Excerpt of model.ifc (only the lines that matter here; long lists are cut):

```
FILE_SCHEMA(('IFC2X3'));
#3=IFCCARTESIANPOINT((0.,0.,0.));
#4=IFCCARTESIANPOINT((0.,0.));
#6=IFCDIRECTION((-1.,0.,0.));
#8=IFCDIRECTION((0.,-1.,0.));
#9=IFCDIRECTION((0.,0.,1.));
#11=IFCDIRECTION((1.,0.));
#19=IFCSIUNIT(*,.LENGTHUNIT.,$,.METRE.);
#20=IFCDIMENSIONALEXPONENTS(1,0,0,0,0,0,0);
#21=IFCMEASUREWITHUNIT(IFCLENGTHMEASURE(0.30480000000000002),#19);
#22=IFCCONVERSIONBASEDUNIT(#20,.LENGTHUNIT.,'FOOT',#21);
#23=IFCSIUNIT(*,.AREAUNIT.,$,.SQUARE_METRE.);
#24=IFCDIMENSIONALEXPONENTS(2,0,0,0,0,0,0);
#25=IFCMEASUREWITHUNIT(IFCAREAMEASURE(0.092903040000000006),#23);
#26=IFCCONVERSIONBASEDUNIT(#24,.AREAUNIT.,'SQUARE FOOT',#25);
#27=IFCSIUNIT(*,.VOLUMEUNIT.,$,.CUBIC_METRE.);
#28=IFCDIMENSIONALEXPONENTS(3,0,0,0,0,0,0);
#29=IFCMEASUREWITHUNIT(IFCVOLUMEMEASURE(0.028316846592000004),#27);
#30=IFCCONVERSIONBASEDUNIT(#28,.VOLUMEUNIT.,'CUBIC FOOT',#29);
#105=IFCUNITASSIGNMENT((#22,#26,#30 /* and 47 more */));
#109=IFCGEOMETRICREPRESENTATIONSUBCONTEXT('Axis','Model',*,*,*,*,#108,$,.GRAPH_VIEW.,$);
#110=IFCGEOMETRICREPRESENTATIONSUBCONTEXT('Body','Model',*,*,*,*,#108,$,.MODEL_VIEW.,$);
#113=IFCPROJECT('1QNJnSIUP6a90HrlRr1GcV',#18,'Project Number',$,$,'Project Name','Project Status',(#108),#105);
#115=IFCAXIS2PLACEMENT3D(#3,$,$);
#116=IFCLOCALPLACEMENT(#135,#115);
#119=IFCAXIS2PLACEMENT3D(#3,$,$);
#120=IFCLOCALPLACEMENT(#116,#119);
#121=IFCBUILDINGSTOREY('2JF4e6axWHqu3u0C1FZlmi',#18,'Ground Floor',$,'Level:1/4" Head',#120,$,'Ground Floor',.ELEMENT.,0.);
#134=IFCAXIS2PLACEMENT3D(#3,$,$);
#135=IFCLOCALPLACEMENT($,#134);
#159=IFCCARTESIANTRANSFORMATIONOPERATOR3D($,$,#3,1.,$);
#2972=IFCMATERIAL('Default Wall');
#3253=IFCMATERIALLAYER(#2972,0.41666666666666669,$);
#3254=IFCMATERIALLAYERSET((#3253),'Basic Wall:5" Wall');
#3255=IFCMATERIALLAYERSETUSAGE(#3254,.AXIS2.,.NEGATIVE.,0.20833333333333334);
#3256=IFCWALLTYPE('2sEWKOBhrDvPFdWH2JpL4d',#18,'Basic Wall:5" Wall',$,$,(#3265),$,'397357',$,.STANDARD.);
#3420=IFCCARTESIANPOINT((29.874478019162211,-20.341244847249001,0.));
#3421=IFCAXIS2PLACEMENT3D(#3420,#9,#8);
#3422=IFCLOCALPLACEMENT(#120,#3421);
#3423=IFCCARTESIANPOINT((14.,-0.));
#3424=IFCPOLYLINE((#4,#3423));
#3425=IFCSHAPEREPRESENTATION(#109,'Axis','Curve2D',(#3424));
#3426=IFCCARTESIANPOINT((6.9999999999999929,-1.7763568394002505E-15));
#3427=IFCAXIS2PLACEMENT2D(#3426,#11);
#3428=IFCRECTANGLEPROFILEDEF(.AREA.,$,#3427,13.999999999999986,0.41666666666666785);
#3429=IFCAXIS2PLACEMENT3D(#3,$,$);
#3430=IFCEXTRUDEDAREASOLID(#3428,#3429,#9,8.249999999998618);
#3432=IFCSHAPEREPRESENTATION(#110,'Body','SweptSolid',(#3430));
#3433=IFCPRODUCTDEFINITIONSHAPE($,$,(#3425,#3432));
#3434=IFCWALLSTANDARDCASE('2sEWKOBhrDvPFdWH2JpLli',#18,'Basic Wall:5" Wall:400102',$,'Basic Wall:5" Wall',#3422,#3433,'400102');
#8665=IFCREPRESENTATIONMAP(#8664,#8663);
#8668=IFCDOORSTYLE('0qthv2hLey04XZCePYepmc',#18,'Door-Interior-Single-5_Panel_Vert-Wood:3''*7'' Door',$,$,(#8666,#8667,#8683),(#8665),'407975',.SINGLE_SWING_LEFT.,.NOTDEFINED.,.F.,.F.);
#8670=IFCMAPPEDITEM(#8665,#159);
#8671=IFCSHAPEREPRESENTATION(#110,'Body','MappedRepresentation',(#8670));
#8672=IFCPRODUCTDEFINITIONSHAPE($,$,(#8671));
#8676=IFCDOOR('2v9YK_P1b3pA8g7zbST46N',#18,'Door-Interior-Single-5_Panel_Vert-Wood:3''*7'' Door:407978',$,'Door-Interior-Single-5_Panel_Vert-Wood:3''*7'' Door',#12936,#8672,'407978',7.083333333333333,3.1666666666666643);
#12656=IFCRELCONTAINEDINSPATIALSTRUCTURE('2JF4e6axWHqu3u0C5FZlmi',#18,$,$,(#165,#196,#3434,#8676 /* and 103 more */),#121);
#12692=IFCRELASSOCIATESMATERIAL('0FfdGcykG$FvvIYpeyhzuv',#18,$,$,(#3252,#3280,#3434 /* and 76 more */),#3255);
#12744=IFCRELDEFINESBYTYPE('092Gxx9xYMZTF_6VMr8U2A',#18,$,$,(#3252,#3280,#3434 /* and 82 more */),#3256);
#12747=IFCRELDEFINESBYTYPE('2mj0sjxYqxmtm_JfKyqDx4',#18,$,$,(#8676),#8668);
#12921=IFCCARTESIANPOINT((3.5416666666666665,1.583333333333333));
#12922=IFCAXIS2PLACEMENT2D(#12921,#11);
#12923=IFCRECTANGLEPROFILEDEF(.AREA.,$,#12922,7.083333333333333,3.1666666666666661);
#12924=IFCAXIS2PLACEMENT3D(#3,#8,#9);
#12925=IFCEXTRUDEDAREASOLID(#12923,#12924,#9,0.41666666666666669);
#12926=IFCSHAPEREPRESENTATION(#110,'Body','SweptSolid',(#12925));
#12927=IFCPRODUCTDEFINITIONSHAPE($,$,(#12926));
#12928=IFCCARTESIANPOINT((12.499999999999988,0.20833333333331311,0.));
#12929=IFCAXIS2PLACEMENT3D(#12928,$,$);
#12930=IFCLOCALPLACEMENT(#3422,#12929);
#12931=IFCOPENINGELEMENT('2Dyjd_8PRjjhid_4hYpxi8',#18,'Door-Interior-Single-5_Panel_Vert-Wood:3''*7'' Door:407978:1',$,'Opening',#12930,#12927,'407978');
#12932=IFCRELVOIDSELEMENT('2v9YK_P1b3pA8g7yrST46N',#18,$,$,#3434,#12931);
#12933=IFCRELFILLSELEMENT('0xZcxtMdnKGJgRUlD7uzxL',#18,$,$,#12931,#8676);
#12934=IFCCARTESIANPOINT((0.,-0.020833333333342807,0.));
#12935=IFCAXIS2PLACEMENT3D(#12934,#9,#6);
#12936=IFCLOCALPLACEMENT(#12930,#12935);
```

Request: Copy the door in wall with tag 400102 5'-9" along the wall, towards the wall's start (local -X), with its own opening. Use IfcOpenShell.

```python
import ifcopenshell
import ifcopenshell.api.feature
import ifcopenshell.api.geometry
import ifcopenshell.api.root
import ifcopenshell.geom
import ifcopenshell.util.element
import ifcopenshell.util.placement
import ifcopenshell.util.shape
import ifcopenshell.util.unit

model = ifcopenshell.open("model.ifc")
unit_scale = ifcopenshell.util.unit.calculate_unit_scale(model)
settings = ifcopenshell.geom.settings()


def volume(element):
    """Net volume in cubic metres, openings subtracted."""
    shape = ifcopenshell.geom.create_shape(settings, element)
    return ifcopenshell.util.shape.get_volume(shape.geometry)


def reuse_history(source, copy):
    """copy_class also copies each property set's owner history, people and application; keep the originals."""
    for rel in copy.IsDefinedBy:
        if rel.is_a("IfcRelDefinesByProperties") and (history := rel.RelatingPropertyDefinition.OwnerHistory):
            rel.RelatingPropertyDefinition.OwnerHistory = source.OwnerHistory
            ifcopenshell.util.element.remove_deep2(model, history)


door = model.by_guid("2v9YK_P1b3pA8g7zbST46N")
opening = door.FillsVoids[0].RelatingOpeningElement
wall = opening.VoidsElements[0].RelatingBuildingElement
before = volume(wall)
shift = ifcopenshell.util.placement.get_local_placement(wall.ObjectPlacement)[:3, 0] * -69 * 0.0254 / unit_scale

# copy_class copies the void relationship, type, container and properties, but no geometry.
new_opening = ifcopenshell.api.root.copy_class(model, product=opening)
new_opening.Representation = ifcopenshell.util.element.copy_deep(
    model, opening.Representation, exclude=["IfcGeometricRepresentationContext", "IfcRepresentationMap"]
)
new_opening.Name = "Door-Interior-Single-5_Panel_Vert-Wood:3'*7' Door"
new_opening.Tag = None
new_door = ifcopenshell.api.root.copy_class(model, product=door)
new_door.Representation = ifcopenshell.util.element.copy_deep(
    model, door.Representation, exclude=["IfcGeometricRepresentationContext", "IfcRepresentationMap"]
)
new_door.Name = "Door-Interior-Single-5_Panel_Vert-Wood:3'*7' Door"
new_door.Tag = None
reuse_history(door, new_door)
fills = ifcopenshell.api.feature.add_filling(model, opening=new_opening, element=new_door)
fills.OwnerHistory = new_door.OwnerHistory  # required in IFC2X3

for old, new in ((opening, new_opening), (door, new_door)):
    matrix = ifcopenshell.util.placement.get_local_placement(old.ObjectPlacement)
    matrix[:3, 3] += shift
    ifcopenshell.api.geometry.edit_object_placement(model, product=new, matrix=matrix, is_si=False)

after = volume(wall)

print(f"wall volume {before:.3f} -> {after:.3f} m3")

model.write("model-out.ifc")
```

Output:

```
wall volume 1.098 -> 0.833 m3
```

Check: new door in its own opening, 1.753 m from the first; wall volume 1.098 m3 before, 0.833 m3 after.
